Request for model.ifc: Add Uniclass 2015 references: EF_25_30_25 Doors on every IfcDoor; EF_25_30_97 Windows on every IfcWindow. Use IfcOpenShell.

First a look at what the model holds.

```python
import ifcopenshell

model = ifcopenshell.open("model.ifc")
print(model.schema)
print("classifications:", [c.Name for c in model.by_type("IfcClassification")])
for ifc_class in ("IfcDoor", "IfcRoof", "IfcStair", "IfcWall", "IfcWindow"):
    print(ifc_class, len(model.by_type(ifc_class)))
```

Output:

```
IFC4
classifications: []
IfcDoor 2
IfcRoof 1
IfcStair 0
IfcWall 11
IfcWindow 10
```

```python
import ifcopenshell
import ifcopenshell.api.classification

model = ifcopenshell.open("model.ifc")

system = ifcopenshell.api.classification.add_classification(model, classification="Uniclass 2015")

codes = {
    "IfcDoor": ("EF_25_30_25", "Doors"),
    "IfcWindow": ("EF_25_30_97", "Windows"),
}
for ifc_class, (code, name) in codes.items():
    products = model.by_type(ifc_class)
    ifcopenshell.api.classification.add_reference(
        model, products=products, classification=system, identification=code, name=name
    )
    print(code, len(products))

model.write("model_rev.ifc")
```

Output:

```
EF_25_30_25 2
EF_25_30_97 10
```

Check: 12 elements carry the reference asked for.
